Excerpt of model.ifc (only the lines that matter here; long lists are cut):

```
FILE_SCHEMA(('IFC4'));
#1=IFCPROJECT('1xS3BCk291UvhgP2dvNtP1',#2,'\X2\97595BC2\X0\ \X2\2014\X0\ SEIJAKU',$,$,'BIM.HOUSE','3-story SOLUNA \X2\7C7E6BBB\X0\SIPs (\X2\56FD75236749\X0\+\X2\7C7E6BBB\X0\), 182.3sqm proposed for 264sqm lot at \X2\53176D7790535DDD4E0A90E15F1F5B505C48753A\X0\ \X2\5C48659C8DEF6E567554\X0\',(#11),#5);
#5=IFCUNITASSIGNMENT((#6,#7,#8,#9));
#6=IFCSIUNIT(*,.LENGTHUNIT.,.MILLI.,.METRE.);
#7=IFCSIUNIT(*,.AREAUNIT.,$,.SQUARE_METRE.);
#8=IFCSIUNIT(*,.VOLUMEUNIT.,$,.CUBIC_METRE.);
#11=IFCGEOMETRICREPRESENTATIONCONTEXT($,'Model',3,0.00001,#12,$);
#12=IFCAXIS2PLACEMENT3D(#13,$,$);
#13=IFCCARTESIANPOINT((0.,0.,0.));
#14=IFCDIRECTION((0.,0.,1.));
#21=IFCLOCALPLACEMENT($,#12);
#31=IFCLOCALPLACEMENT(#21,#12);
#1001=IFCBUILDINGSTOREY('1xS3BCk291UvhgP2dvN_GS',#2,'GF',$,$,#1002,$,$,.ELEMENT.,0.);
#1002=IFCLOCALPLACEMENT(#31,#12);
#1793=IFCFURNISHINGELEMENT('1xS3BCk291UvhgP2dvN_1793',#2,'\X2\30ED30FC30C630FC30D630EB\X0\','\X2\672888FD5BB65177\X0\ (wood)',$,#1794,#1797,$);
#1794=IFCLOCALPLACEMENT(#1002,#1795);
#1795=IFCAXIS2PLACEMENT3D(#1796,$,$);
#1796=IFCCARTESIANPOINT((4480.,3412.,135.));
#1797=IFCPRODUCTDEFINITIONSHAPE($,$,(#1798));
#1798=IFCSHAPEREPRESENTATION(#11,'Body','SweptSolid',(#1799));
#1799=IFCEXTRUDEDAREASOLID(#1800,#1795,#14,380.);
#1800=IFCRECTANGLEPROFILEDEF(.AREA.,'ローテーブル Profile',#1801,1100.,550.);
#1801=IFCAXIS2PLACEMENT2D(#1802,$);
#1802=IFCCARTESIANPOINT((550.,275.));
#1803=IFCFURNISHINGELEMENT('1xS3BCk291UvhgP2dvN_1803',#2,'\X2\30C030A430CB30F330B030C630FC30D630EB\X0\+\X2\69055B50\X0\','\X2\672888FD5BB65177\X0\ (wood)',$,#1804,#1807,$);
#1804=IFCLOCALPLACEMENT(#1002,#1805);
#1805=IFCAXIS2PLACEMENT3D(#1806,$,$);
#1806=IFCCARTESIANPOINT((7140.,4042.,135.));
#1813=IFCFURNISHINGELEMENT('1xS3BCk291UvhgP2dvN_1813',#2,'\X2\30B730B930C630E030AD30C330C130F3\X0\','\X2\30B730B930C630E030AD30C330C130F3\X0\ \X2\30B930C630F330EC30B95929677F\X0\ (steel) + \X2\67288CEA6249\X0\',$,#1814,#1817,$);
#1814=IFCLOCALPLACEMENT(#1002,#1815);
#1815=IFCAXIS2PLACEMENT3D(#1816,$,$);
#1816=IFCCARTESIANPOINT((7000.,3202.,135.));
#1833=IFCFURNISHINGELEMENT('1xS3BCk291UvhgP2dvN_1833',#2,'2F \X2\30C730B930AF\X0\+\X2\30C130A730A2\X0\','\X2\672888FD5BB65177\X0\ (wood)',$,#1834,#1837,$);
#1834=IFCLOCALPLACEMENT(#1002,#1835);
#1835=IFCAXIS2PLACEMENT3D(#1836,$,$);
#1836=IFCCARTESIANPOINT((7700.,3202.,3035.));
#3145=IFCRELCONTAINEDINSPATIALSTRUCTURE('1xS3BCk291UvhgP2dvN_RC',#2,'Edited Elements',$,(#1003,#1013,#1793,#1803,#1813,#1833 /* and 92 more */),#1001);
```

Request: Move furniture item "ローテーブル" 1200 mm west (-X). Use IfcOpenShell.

```python
import ifcopenshell
import ifcopenshell.api.geometry
import ifcopenshell.util.placement

model = ifcopenshell.open("model.ifc")

item = model.by_guid("1xS3BCk291UvhgP2dvN_1793")
matrix = ifcopenshell.util.placement.get_local_placement(item.ObjectPlacement)
matrix[0, 3] -= 1200.0
ifcopenshell.api.geometry.edit_object_placement(model, product=item, matrix=matrix, is_si=False)

print(ifcopenshell.util.placement.get_local_placement(item.ObjectPlacement).round(3) + 0.0)

model.write("model_rev.ifc")
```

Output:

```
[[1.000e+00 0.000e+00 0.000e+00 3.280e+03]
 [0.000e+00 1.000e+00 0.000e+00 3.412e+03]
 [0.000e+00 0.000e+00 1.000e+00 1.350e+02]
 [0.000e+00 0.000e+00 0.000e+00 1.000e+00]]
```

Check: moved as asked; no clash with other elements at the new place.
